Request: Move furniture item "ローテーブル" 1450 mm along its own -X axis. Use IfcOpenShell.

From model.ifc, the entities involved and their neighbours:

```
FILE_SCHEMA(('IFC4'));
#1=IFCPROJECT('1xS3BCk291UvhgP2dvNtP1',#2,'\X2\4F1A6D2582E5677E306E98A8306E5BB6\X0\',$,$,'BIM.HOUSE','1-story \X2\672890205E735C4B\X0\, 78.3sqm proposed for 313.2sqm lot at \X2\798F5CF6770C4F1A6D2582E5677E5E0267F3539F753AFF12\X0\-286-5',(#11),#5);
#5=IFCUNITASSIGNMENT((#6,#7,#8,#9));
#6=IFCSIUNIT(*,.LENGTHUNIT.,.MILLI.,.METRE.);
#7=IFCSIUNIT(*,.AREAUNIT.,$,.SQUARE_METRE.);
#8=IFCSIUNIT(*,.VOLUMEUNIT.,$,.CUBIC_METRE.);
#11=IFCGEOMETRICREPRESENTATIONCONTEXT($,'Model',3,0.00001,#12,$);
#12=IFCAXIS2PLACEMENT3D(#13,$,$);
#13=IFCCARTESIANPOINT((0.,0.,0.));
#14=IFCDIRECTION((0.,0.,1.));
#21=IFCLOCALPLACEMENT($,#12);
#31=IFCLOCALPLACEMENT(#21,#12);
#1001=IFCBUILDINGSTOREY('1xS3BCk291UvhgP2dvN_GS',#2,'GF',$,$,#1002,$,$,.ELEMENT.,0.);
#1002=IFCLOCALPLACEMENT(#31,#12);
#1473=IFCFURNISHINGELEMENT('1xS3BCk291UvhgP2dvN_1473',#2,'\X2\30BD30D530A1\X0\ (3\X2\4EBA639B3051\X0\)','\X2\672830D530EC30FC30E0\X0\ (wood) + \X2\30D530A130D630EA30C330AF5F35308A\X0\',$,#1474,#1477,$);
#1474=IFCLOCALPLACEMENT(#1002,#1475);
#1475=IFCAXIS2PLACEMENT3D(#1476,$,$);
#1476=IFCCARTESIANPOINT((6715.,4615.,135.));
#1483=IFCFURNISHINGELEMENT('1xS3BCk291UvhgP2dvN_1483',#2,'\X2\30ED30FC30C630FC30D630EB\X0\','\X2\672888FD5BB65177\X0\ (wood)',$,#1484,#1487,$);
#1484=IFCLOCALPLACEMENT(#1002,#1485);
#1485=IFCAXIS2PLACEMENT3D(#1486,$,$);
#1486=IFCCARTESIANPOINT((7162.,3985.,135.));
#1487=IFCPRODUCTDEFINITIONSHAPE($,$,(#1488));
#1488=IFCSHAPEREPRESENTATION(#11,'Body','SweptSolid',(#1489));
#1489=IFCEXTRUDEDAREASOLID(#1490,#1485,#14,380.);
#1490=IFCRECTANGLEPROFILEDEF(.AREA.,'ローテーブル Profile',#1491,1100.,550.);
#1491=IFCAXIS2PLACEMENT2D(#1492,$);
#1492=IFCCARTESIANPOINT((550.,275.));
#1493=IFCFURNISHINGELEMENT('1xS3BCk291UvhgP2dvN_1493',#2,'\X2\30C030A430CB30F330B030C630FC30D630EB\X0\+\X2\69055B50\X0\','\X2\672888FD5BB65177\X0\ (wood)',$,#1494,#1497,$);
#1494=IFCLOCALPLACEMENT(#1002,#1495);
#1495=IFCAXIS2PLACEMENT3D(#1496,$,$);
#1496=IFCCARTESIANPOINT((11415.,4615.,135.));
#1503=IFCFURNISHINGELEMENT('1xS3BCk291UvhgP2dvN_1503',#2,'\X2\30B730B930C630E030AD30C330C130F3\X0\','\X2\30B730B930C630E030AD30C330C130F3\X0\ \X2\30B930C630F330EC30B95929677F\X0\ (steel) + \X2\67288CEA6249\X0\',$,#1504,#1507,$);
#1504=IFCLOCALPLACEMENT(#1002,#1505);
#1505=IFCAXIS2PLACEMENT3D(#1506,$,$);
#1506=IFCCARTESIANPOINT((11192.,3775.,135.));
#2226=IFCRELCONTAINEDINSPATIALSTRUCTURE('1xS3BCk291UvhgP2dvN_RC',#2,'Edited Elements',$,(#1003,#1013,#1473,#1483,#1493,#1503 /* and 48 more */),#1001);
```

```python
import ifcopenshell
import ifcopenshell.api.geometry
import ifcopenshell.util.placement
import ifcopenshell.util.unit

model = ifcopenshell.open("model.ifc")
unit_scale = ifcopenshell.util.unit.calculate_unit_scale(model)

item = model.by_guid("1xS3BCk291UvhgP2dvN_1483")
matrix = ifcopenshell.util.placement.get_local_placement(item.ObjectPlacement)
matrix[:3, 3] -= matrix[:3, 0] * 1.45 / unit_scale
ifcopenshell.api.geometry.edit_object_placement(model, product=item, matrix=matrix, is_si=False)

print(ifcopenshell.util.placement.get_local_placement(item.ObjectPlacement).round(3) + 0.0)

model.write("model_v2.ifc")
```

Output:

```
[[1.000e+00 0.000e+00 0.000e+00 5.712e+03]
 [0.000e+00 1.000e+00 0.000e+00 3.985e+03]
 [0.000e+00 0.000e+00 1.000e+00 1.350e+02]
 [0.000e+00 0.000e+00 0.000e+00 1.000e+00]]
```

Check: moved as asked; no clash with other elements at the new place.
